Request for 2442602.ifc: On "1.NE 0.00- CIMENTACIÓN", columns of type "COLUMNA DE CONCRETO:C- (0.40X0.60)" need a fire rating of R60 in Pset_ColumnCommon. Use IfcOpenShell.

First a look at what the model holds.

```python
import ifcopenshell
import ifcopenshell.util.element

model = ifcopenshell.open("2442602.ifc")
print(model.schema)
storey = next(s for s in model.by_type("IfcBuildingStorey") if s.Name == "1.NE 0.00- CIMENTACIÓN")
columns = [e for e in ifcopenshell.util.element.get_decomposition(storey) if e.is_a("IfcColumn")]
seen = {}
for e in columns:
    element_type = ifcopenshell.util.element.get_type(e)
    key = (element_type.Name if element_type != e and element_type else None, ifcopenshell.util.element.get_pset(e, "Pset_ColumnCommon", "FireRating"))
    seen[key] = seen.get(key, 0) + 1
for (name, value), count in sorted(seen.items(), key=str):
    print(count, "x", name, "|", value)
```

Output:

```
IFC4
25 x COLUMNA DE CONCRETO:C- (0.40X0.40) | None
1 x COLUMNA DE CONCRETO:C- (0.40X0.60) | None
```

```python
import ifcopenshell
import ifcopenshell.api.pset
import ifcopenshell.util.element

model = ifcopenshell.open("2442602.ifc")

storey = next(s for s in model.by_type("IfcBuildingStorey") if s.Name == "1.NE 0.00- CIMENTACIÓN")
columns = [e for e in ifcopenshell.util.element.get_decomposition(storey) if e.is_a("IfcColumn")]

count = 0
for e in columns:
    element_type = ifcopenshell.util.element.get_type(e)
    if element_type in (None, e) or element_type.Name != "COLUMNA DE CONCRETO:C- (0.40X0.60)":
        continue
    # add_pset returns the element's existing set when there is one.
    pset = ifcopenshell.api.pset.add_pset(model, product=e, name="Pset_ColumnCommon")
    ifcopenshell.api.pset.edit_pset(model, pset=pset, properties={"FireRating": "R60"})
    count += 1

print(count, "columns updated")

model.write("2442602_edited.ifc")
```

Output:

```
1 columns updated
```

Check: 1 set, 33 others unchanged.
